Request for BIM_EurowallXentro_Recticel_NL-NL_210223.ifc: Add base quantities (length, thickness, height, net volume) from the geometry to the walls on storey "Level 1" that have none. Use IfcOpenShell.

First a look at what the model holds.

```python
import ifcopenshell
import ifcopenshell.util.element
import ifcopenshell.util.unit

model = ifcopenshell.open("BIM_EurowallXentro_Recticel_NL-NL_210223.ifc")
print(model.schema)
for unit_type in ("LENGTHUNIT", "AREAUNIT", "VOLUMEUNIT"):
    print(unit_type, ifcopenshell.util.unit.calculate_unit_scale(model, unit_type))
storey = next(s for s in model.by_type("IfcBuildingStorey") if s.Name == "Level 1")
walls = [e for e in ifcopenshell.util.element.get_decomposition(storey) if e.is_a("IfcWall")]
for e in sorted(walls, key=lambda e: e.id()):
    print(e.id(), e.is_a(), e.Name, list(ifcopenshell.util.element.get_psets(e, qtos_only=True)), sep=" | ")
```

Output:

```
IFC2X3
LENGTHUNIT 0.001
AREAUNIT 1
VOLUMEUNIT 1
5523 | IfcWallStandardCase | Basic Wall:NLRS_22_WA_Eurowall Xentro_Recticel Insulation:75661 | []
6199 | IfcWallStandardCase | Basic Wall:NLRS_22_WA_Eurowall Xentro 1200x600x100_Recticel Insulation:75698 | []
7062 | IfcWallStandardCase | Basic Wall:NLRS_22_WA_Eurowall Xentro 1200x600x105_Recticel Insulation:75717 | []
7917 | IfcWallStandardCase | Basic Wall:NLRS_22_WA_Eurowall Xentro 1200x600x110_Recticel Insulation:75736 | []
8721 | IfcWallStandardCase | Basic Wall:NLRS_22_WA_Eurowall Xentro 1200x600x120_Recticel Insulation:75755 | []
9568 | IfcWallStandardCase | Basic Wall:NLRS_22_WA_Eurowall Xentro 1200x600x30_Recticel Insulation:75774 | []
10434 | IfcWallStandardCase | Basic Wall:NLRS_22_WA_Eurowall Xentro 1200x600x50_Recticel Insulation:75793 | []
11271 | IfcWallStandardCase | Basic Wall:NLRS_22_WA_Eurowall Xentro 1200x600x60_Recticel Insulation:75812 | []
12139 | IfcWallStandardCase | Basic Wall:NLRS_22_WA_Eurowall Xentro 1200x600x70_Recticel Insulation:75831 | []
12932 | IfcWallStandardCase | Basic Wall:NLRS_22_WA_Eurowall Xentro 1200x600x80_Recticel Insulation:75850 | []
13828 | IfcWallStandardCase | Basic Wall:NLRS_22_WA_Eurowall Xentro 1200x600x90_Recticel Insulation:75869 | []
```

```python
import ifcopenshell
import ifcopenshell.api.pset
import ifcopenshell.geom
import ifcopenshell.util.element
import ifcopenshell.util.shape
import ifcopenshell.util.unit

model = ifcopenshell.open("BIM_EurowallXentro_Recticel_NL-NL_210223.ifc")
unit_scale = ifcopenshell.util.unit.calculate_unit_scale(model)
volume_scale = ifcopenshell.util.unit.calculate_unit_scale(model, "VOLUMEUNIT")
settings = ifcopenshell.geom.settings()

storey = next(s for s in model.by_type("IfcBuildingStorey") if s.Name == "Level 1")
walls = [e for e in ifcopenshell.util.element.get_decomposition(storey) if e.is_a("IfcWall")]

for e in sorted(walls, key=lambda e: e.id()):
    if ifcopenshell.util.element.get_psets(e, qtos_only=True, should_inherit=False):
        continue
    # Geometry comes back in metres, in the element's own axes.
    shape = ifcopenshell.geom.create_shape(settings, e)
    values = {
        "Length": ifcopenshell.util.shape.get_x(shape.geometry) / unit_scale,
        "Width": ifcopenshell.util.shape.get_y(shape.geometry) / unit_scale,
        "Height": ifcopenshell.util.shape.get_z(shape.geometry) / unit_scale,
        "NetVolume": ifcopenshell.util.shape.get_volume(shape.geometry) / volume_scale,
    }
    qto = ifcopenshell.api.pset.add_qto(model, product=e, name="BaseQuantities")
    ifcopenshell.api.pset.edit_qto(model, qto=qto, properties=values)
    print(e.id(), {k: round(v, 3) for k, v in values.items()})

model.write("BIM_EurowallXentro_Recticel_NL-NL_210223_updated.ifc")
```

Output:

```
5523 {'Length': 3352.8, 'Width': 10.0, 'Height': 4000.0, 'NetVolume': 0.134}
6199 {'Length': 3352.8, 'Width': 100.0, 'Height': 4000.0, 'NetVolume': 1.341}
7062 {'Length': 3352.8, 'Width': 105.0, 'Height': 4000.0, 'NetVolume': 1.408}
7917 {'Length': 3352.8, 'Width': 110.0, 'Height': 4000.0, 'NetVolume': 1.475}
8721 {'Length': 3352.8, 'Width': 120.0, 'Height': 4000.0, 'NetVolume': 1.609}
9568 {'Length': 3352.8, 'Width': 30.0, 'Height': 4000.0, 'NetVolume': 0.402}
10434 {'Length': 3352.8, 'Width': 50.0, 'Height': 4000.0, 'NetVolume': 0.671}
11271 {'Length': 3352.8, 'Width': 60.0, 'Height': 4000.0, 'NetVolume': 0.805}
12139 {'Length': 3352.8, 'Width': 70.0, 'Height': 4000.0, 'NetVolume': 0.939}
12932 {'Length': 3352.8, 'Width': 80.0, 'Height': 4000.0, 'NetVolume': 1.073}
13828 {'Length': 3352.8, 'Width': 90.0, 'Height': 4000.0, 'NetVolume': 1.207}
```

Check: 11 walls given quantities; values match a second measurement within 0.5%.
